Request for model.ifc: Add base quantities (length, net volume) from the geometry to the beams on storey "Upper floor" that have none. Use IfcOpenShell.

First a look at what the model holds.

```python
import ifcopenshell
import ifcopenshell.util.element
import ifcopenshell.util.unit

model = ifcopenshell.open("model.ifc")
print(model.schema)
for unit_type in ("LENGTHUNIT", "AREAUNIT", "VOLUMEUNIT"):
    print(unit_type, ifcopenshell.util.unit.calculate_unit_scale(model, unit_type))
storey = next(s for s in model.by_type("IfcBuildingStorey") if s.Name == "Upper floor")
beams = [e for e in ifcopenshell.util.element.get_decomposition(storey) if e.is_a("IfcBeam")]
for e in sorted(beams, key=lambda e: e.id()):
    print(e.id(), e.is_a(), e.Name, list(ifcopenshell.util.element.get_psets(e, qtos_only=True)), sep=" | ")
```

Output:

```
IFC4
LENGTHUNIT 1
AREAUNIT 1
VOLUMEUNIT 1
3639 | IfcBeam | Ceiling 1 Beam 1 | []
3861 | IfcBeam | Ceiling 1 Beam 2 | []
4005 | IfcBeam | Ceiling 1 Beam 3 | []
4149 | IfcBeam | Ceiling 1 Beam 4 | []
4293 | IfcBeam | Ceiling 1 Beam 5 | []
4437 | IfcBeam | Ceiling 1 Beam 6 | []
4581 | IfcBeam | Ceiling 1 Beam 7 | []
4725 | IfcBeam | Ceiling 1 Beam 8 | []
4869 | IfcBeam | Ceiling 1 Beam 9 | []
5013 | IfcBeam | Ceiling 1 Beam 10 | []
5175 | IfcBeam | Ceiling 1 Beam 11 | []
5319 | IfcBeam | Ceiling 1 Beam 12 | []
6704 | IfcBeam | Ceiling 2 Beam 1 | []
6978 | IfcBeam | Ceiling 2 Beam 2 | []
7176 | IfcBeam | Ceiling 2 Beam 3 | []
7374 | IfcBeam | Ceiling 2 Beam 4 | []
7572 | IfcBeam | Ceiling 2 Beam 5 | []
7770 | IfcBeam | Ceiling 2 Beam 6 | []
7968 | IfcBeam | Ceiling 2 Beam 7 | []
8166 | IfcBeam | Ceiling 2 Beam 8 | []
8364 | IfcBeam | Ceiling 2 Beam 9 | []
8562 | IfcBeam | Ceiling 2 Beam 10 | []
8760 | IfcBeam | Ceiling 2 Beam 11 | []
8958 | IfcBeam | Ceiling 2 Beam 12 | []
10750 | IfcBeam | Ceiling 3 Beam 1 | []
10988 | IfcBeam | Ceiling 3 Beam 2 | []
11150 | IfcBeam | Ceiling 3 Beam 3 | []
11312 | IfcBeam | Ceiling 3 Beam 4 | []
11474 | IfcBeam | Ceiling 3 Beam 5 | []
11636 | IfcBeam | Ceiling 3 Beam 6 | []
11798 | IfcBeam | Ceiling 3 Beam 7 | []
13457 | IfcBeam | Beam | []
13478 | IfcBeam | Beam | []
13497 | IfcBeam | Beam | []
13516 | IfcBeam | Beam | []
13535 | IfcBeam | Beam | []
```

```python
import ifcopenshell
import ifcopenshell.api.pset
import ifcopenshell.geom
import ifcopenshell.util.element
import ifcopenshell.util.shape
import ifcopenshell.util.unit

model = ifcopenshell.open("model.ifc")
unit_scale = ifcopenshell.util.unit.calculate_unit_scale(model)
volume_scale = ifcopenshell.util.unit.calculate_unit_scale(model, "VOLUMEUNIT")
settings = ifcopenshell.geom.settings()

storey = next(s for s in model.by_type("IfcBuildingStorey") if s.Name == "Upper floor")
beams = [e for e in ifcopenshell.util.element.get_decomposition(storey) if e.is_a("IfcBeam")]

for e in sorted(beams, key=lambda e: e.id()):
    if ifcopenshell.util.element.get_psets(e, qtos_only=True, should_inherit=False):
        continue
    # Geometry comes back in metres, in the element's own axes.
    shape = ifcopenshell.geom.create_shape(settings, e)
    values = {
        "Length": ifcopenshell.util.shape.get_max_xyz(shape.geometry) / unit_scale,
        "NetVolume": ifcopenshell.util.shape.get_volume(shape.geometry) / volume_scale,
    }
    qto = ifcopenshell.api.pset.add_qto(model, product=e, name="Qto_BeamBaseQuantities")
    ifcopenshell.api.pset.edit_qto(model, qto=qto, properties=values)
    print(e.id(), {k: round(v, 3) for k, v in values.items()})

model.write("model-out.ifc")
```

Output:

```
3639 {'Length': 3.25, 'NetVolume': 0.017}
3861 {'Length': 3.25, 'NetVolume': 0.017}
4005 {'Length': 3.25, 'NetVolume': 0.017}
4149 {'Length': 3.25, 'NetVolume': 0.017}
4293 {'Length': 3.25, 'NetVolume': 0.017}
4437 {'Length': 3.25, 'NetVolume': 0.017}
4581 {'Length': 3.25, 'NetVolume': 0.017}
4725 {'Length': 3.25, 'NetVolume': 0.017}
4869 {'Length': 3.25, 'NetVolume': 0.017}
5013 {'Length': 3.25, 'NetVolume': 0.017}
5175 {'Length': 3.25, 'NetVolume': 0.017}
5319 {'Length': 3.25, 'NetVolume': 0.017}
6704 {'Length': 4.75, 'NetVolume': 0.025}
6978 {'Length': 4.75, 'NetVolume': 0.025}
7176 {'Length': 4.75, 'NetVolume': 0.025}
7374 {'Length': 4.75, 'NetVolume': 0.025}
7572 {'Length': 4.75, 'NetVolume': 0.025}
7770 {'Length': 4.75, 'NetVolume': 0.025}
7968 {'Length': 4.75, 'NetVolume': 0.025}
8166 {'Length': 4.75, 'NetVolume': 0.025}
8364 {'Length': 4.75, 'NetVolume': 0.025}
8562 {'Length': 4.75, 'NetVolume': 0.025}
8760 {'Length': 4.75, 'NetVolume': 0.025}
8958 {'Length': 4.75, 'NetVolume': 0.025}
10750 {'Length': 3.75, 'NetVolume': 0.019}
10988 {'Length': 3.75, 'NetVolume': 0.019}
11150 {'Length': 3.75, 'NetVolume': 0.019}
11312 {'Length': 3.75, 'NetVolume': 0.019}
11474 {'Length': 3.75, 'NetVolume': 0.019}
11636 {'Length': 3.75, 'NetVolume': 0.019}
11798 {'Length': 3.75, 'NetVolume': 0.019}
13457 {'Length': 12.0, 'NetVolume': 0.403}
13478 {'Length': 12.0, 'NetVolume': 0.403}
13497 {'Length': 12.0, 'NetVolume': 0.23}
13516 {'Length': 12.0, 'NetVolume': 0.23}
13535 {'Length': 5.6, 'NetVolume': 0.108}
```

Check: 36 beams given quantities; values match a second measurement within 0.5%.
